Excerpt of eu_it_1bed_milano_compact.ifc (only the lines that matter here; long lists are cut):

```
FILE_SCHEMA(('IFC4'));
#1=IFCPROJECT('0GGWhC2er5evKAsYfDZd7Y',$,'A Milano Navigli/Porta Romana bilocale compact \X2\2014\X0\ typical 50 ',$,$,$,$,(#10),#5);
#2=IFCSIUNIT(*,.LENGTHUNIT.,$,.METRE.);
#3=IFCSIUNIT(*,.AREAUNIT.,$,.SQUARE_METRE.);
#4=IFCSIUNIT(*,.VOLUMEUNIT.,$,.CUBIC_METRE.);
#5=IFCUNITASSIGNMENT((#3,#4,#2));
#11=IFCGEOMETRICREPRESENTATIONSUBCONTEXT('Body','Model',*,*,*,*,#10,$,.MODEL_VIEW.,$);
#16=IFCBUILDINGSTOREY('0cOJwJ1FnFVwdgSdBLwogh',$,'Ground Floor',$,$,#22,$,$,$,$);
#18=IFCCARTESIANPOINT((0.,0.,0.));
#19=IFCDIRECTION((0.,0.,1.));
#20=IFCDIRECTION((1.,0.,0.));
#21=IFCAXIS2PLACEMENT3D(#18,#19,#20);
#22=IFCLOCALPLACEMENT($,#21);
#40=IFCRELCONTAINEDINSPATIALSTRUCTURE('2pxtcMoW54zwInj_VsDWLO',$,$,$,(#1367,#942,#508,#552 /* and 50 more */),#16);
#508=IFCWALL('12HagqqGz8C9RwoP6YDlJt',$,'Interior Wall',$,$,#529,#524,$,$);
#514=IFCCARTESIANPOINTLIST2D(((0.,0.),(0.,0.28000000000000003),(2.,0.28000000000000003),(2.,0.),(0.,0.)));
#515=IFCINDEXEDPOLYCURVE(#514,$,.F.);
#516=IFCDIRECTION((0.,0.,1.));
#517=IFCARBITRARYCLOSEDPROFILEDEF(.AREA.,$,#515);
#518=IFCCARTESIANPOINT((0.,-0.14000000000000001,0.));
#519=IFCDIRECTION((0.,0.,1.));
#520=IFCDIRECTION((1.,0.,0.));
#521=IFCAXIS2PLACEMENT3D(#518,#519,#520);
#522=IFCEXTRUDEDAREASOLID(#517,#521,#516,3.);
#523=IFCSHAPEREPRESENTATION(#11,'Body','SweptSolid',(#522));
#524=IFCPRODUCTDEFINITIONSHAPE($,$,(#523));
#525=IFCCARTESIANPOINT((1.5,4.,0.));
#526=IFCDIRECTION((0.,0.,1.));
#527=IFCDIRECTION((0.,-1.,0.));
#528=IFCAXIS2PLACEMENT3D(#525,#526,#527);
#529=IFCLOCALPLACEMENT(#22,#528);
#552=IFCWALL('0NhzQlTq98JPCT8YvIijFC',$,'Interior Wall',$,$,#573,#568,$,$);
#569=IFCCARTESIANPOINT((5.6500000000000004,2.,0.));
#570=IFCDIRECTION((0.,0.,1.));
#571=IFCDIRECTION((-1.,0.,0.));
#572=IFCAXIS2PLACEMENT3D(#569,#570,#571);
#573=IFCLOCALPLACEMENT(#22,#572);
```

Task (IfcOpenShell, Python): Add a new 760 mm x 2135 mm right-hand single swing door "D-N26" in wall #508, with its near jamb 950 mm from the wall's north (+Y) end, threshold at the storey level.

```python
import numpy as np
import ifcopenshell
import ifcopenshell.api.feature
import ifcopenshell.api.geometry
import ifcopenshell.api.root
import ifcopenshell.api.spatial
import ifcopenshell.geom
import ifcopenshell.util.element
import ifcopenshell.util.placement
import ifcopenshell.util.representation
import ifcopenshell.util.shape
import ifcopenshell.util.unit

model = ifcopenshell.open("eu_it_1bed_milano_compact.ifc")
unit_scale = ifcopenshell.util.unit.calculate_unit_scale(model)
settings = ifcopenshell.geom.settings()


def volume(element):
    """Net volume in cubic metres, openings subtracted."""
    shape = ifcopenshell.geom.create_shape(settings, element)
    return ifcopenshell.util.shape.get_volume(shape.geometry)


wall = model.by_guid("12HagqqGz8C9RwoP6YDlJt")
storey = ifcopenshell.util.element.get_container(wall, ifc_class="IfcBuildingStorey")
context = ifcopenshell.util.representation.get_context(model, "Model", "Body", "MODEL_VIEW")
before = volume(wall)

width, height, from_end, sill = 0.76, 2.135, 0.95, 0.0  # metres

# The wall runs along its own X axis, and the end named is its -X end.
wall_shape = ifcopenshell.geom.create_shape(settings, wall)
x, y, z = ifcopenshell.util.shape.get_vertices(wall_shape.geometry).T
start = x.min() + from_end
face, thickness = float(y.min()), float(y.max() - y.min())
wall_matrix = ifcopenshell.util.placement.get_local_placement(wall.ObjectPlacement)
level = ifcopenshell.util.placement.get_local_placement(storey.ObjectPlacement)[2, 3]


def in_wall(x, y):
    """Placement at x, y metres in the wall's axes, at sill height."""
    matrix = wall_matrix.copy()
    matrix[:, 3] = wall_matrix @ np.array([x / unit_scale, y / unit_scale, 0.0, 1.0])
    matrix[2, 3] = level + sill / unit_scale
    return matrix


# Opening: a box that overshoots both wall faces by 50 mm.
opening = ifcopenshell.api.root.create_entity(model, ifc_class="IfcOpeningElement", predefined_type="OPENING")
box = ifcopenshell.api.geometry.add_wall_representation(
    model, context=context, length=width, height=height, thickness=thickness + 0.1
)
ifcopenshell.api.geometry.assign_representation(model, product=opening, representation=box)
ifcopenshell.api.geometry.edit_object_placement(model, product=opening, matrix=in_wall(start, face - 0.05), is_si=False)
ifcopenshell.api.feature.add_feature(model, feature=opening, element=wall)

door = ifcopenshell.api.root.create_entity(model, ifc_class="IfcDoor", name="D-N26", predefined_type="DOOR")
door.OverallWidth, door.OverallHeight = width / unit_scale, height / unit_scale
door.OperationType = "SINGLE_SWING_RIGHT"
body = ifcopenshell.api.geometry.add_door_representation(
    model,
    context=context,
    overall_width=door.OverallWidth,
    overall_height=door.OverallHeight,
    operation_type="SINGLE_SWING_RIGHT",
    lining_properties={"LiningDepth": thickness / unit_scale, "ThresholdDepth": thickness / unit_scale},
)
ifcopenshell.api.geometry.assign_representation(model, product=door, representation=body)
ifcopenshell.api.spatial.assign_container(model, products=[door], relating_structure=storey)
ifcopenshell.api.feature.add_filling(model, opening=opening, element=door)

# The lining spans the wall, so the door starts at the wall face.
ifcopenshell.api.geometry.edit_object_placement(model, product=door, matrix=in_wall(start, face), is_si=False)

after = volume(wall)

print(f"wall volume {before:.3f} -> {after:.3f} m3")

model.write("eu_it_1bed_milano_compact_updated.ifc")
```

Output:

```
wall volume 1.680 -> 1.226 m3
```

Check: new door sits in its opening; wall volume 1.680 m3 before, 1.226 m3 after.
